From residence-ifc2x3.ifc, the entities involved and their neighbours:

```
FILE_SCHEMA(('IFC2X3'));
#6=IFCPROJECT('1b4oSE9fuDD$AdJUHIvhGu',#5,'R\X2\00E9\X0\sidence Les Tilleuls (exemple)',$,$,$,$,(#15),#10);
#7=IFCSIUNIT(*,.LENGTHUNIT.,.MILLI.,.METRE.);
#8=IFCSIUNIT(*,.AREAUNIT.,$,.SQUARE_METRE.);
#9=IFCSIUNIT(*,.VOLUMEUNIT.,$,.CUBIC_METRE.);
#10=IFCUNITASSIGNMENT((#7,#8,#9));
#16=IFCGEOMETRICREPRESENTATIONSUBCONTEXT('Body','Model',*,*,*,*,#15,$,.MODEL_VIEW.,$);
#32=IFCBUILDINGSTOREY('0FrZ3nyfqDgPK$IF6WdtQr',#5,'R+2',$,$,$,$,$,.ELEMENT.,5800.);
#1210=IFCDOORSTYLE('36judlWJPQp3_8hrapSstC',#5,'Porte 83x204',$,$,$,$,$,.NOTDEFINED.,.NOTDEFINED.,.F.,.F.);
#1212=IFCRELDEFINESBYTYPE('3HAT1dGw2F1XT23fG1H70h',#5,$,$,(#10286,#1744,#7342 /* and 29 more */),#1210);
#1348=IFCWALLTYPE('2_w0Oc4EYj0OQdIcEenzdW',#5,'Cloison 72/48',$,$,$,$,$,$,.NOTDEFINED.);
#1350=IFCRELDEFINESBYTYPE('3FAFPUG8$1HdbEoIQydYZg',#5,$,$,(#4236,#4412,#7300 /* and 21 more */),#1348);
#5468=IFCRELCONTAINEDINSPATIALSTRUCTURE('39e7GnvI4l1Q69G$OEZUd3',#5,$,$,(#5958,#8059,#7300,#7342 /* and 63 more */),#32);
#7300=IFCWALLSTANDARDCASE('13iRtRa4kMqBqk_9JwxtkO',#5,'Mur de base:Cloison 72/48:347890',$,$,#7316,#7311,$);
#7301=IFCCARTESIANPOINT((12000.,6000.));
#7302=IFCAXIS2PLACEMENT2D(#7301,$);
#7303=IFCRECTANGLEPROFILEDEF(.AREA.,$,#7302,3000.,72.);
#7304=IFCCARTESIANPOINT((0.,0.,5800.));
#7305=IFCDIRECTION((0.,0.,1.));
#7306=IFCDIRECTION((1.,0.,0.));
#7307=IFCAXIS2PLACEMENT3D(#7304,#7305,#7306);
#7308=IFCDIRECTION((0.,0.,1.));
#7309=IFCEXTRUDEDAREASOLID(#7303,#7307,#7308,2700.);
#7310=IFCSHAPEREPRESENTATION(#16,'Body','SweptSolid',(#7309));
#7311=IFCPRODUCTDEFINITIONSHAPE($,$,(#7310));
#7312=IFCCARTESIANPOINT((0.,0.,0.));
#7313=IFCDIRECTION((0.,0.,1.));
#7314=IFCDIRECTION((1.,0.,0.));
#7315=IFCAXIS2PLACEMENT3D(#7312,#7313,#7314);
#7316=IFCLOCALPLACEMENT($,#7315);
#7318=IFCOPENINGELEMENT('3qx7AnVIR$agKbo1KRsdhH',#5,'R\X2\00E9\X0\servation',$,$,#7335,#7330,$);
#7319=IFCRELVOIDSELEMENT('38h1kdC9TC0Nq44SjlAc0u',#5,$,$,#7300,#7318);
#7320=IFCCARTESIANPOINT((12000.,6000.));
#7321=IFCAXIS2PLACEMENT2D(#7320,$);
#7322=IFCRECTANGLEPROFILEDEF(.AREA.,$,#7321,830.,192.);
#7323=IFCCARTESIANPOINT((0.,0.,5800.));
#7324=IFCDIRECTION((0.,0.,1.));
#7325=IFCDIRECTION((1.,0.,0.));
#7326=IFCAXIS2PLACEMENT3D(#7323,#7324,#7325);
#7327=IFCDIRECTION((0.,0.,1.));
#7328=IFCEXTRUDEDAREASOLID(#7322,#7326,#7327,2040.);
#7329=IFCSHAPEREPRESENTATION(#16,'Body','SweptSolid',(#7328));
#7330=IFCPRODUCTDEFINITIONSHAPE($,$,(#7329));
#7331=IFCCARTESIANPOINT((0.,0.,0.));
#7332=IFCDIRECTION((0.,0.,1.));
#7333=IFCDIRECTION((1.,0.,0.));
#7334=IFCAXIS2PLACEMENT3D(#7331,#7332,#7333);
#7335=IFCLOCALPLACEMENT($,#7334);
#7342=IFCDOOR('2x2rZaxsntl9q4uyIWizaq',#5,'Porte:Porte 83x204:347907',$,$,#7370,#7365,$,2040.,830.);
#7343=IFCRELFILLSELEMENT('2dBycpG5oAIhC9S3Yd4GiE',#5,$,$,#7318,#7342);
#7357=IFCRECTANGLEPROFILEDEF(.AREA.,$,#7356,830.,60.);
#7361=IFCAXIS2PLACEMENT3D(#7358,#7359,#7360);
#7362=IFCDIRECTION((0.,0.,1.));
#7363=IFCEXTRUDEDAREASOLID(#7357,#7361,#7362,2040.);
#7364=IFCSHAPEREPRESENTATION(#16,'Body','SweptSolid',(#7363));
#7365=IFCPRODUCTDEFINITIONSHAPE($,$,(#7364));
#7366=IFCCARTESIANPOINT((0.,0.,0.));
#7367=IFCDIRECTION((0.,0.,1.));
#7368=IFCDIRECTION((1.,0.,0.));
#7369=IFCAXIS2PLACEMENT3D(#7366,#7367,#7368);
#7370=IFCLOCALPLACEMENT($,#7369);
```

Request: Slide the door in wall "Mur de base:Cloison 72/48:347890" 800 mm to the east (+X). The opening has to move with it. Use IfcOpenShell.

```python
import ifcopenshell
import ifcopenshell.api.geometry
import ifcopenshell.util.placement
import ifcopenshell.util.unit

model = ifcopenshell.open("residence-ifc2x3.ifc")
unit_scale = ifcopenshell.util.unit.calculate_unit_scale(model)

door = model.by_guid("2x2rZaxsntl9q4uyIWizaq")
opening = door.FillsVoids[0].RelatingOpeningElement
wall = opening.VoidsElements[0].RelatingBuildingElement

wall_matrix = ifcopenshell.util.placement.get_local_placement(wall.ObjectPlacement)
shift = wall_matrix[:3, 0] * 0.8 / unit_scale
before = ifcopenshell.util.placement.get_local_placement(door.ObjectPlacement)[:3, 3].copy()

# The door is not placed relative to its opening, so move both.
for product in (opening, door):
    matrix = ifcopenshell.util.placement.get_local_placement(product.ObjectPlacement)
    matrix[:3, 3] += shift
    ifcopenshell.api.geometry.edit_object_placement(model, product=product, matrix=matrix, is_si=False)

after = ifcopenshell.util.placement.get_local_placement(door.ObjectPlacement)[:3, 3]
print("door moved by", (after - before).round(3) + 0.0)

model.write("residence-ifc2x3_updated.ifc")
```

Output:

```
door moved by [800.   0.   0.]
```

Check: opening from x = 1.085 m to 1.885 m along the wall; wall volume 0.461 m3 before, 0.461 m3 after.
